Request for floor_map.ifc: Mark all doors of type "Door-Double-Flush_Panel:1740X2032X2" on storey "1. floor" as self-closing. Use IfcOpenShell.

First a look at what the model holds.

```python
import ifcopenshell
import ifcopenshell.util.element

model = ifcopenshell.open("floor_map.ifc")
print(model.schema)
storey = next(s for s in model.by_type("IfcBuildingStorey") if s.Name == "1. floor")
doors = [e for e in ifcopenshell.util.element.get_decomposition(storey) if e.is_a("IfcDoor")]
seen = {}
for e in doors:
    element_type = ifcopenshell.util.element.get_type(e)
    key = (element_type.Name if element_type != e and element_type else None, ifcopenshell.util.element.get_pset(e, "Pset_DoorCommon", "SelfClosing"))
    seen[key] = seen.get(key, 0) + 1
for (name, value), count in sorted(seen.items(), key=str):
    print(count, "x", name, "|", value)
```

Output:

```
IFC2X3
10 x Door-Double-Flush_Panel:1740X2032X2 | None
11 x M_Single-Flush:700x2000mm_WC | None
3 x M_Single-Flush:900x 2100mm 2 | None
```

```python
import ifcopenshell
import ifcopenshell.api.pset
import ifcopenshell.util.element

model = ifcopenshell.open("floor_map.ifc")

storey = next(s for s in model.by_type("IfcBuildingStorey") if s.Name == "1. floor")
doors = [e for e in ifcopenshell.util.element.get_decomposition(storey) if e.is_a("IfcDoor")]

count = 0
for e in doors:
    element_type = ifcopenshell.util.element.get_type(e)
    if element_type in (None, e) or element_type.Name != "Door-Double-Flush_Panel:1740X2032X2":
        continue
    # add_pset returns the element's existing set when there is one.
    pset = ifcopenshell.api.pset.add_pset(model, product=e, name="Pset_DoorCommon")
    ifcopenshell.api.pset.edit_pset(model, pset=pset, properties={"SelfClosing": True})
    count += 1

print(count, "doors updated")

model.write("floor_map_edited.ifc")
```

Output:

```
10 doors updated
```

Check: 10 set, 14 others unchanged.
